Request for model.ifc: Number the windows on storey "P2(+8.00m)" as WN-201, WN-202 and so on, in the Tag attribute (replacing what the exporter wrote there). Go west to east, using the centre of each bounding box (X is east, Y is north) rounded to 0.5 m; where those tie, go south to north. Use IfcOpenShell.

First a look at what the model holds.

```python
import ifcopenshell
import ifcopenshell.util.element
import ifcopenshell.util.placement

model = ifcopenshell.open("model.ifc")
print(model.schema)
storey = next(s for s in model.by_type("IfcBuildingStorey") if s.Name == "P2(+8.00m)")
windows = [e for e in ifcopenshell.util.element.get_decomposition(storey) if e.is_a("IfcWindow")]
for e in sorted(windows, key=lambda e: e.id()):
    origin = ifcopenshell.util.placement.get_local_placement(e.ObjectPlacement)[:3, 3]
    print(e.id(), e.Tag, e.Name, origin.round(2) + 0.0, sep=" | ")
```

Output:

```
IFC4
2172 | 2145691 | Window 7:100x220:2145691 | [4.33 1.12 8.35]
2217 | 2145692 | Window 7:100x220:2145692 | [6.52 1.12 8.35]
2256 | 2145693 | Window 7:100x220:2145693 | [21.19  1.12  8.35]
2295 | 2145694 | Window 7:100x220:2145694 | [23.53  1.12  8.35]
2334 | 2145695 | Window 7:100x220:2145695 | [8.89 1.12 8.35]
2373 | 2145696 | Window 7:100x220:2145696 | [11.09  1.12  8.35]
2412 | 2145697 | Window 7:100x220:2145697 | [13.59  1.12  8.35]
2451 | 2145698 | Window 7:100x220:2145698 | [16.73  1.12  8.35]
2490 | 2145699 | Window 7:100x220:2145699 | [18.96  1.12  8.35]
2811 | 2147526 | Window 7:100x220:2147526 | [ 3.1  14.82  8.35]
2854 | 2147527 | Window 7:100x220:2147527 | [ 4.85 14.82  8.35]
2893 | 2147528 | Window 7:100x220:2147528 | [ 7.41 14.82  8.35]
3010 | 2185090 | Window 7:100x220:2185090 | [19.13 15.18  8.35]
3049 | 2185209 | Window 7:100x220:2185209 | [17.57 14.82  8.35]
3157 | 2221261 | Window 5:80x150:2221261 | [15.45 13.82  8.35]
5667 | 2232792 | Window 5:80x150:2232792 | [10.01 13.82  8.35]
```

```python
import ifcopenshell
import ifcopenshell.geom
import ifcopenshell.util.element
import ifcopenshell.util.shape

model = ifcopenshell.open("model.ifc")
settings = ifcopenshell.geom.settings()
settings.set("use-world-coords", True)


def centre(element):
    shape = ifcopenshell.geom.create_shape(settings, element)
    return ifcopenshell.util.shape.get_bbox_centroid(shape.geometry)


storey = next(s for s in model.by_type("IfcBuildingStorey") if s.Name == "P2(+8.00m)")
windows = [e for e in ifcopenshell.util.element.get_decomposition(storey) if e.is_a("IfcWindow")]

# Insertion points can sit at a corner or the storey origin, so sort by the geometry (in metres).
centres = {e: centre(e) for e in windows}
windows.sort(key=lambda e: (round(centres[e][0] / 0.5), centres[e][1]))

for i, e in enumerate(windows, start=1):
    number = f"WN-2{i:02d}"
    e.Tag = number
    print(e.id(), number)

model.write("model-out.ifc")
```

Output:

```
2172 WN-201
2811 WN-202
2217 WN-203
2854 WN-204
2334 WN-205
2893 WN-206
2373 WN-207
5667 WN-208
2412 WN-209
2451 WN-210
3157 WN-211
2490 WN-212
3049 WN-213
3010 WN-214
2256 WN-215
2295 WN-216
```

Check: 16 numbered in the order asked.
